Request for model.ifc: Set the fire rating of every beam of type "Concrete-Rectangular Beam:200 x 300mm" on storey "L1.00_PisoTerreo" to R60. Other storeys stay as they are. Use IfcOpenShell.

First a look at what the model holds.

```python
import ifcopenshell
import ifcopenshell.util.element

model = ifcopenshell.open("model.ifc")
print(model.schema)
storey = next(s for s in model.by_type("IfcBuildingStorey") if s.Name == "L1.00_PisoTerreo")
beams = [e for e in ifcopenshell.util.element.get_decomposition(storey) if e.is_a("IfcBeam")]
seen = {}
for e in beams:
    element_type = ifcopenshell.util.element.get_type(e)
    key = (element_type.Name if element_type != e and element_type else None, ifcopenshell.util.element.get_pset(e, "Pset_BeamCommon", "FireRating"))
    seen[key] = seen.get(key, 0) + 1
for (name, value), count in sorted(seen.items(), key=str):
    print(count, "x", name, "|", value)
```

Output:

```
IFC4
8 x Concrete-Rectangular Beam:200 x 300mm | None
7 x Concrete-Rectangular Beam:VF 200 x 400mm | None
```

```python
import ifcopenshell
import ifcopenshell.api.pset
import ifcopenshell.util.element

model = ifcopenshell.open("model.ifc")

storey = next(s for s in model.by_type("IfcBuildingStorey") if s.Name == "L1.00_PisoTerreo")
beams = [e for e in ifcopenshell.util.element.get_decomposition(storey) if e.is_a("IfcBeam")]

count = 0
for e in beams:
    element_type = ifcopenshell.util.element.get_type(e)
    if element_type in (None, e) or element_type.Name != "Concrete-Rectangular Beam:200 x 300mm":
        continue
    # add_pset returns the element's existing set when there is one.
    pset = ifcopenshell.api.pset.add_pset(model, product=e, name="Pset_BeamCommon")
    ifcopenshell.api.pset.edit_pset(model, pset=pset, properties={"FireRating": "R60"})
    count += 1

print(count, "beams updated")

model.write("model-out.ifc")
```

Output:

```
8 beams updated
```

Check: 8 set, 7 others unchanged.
